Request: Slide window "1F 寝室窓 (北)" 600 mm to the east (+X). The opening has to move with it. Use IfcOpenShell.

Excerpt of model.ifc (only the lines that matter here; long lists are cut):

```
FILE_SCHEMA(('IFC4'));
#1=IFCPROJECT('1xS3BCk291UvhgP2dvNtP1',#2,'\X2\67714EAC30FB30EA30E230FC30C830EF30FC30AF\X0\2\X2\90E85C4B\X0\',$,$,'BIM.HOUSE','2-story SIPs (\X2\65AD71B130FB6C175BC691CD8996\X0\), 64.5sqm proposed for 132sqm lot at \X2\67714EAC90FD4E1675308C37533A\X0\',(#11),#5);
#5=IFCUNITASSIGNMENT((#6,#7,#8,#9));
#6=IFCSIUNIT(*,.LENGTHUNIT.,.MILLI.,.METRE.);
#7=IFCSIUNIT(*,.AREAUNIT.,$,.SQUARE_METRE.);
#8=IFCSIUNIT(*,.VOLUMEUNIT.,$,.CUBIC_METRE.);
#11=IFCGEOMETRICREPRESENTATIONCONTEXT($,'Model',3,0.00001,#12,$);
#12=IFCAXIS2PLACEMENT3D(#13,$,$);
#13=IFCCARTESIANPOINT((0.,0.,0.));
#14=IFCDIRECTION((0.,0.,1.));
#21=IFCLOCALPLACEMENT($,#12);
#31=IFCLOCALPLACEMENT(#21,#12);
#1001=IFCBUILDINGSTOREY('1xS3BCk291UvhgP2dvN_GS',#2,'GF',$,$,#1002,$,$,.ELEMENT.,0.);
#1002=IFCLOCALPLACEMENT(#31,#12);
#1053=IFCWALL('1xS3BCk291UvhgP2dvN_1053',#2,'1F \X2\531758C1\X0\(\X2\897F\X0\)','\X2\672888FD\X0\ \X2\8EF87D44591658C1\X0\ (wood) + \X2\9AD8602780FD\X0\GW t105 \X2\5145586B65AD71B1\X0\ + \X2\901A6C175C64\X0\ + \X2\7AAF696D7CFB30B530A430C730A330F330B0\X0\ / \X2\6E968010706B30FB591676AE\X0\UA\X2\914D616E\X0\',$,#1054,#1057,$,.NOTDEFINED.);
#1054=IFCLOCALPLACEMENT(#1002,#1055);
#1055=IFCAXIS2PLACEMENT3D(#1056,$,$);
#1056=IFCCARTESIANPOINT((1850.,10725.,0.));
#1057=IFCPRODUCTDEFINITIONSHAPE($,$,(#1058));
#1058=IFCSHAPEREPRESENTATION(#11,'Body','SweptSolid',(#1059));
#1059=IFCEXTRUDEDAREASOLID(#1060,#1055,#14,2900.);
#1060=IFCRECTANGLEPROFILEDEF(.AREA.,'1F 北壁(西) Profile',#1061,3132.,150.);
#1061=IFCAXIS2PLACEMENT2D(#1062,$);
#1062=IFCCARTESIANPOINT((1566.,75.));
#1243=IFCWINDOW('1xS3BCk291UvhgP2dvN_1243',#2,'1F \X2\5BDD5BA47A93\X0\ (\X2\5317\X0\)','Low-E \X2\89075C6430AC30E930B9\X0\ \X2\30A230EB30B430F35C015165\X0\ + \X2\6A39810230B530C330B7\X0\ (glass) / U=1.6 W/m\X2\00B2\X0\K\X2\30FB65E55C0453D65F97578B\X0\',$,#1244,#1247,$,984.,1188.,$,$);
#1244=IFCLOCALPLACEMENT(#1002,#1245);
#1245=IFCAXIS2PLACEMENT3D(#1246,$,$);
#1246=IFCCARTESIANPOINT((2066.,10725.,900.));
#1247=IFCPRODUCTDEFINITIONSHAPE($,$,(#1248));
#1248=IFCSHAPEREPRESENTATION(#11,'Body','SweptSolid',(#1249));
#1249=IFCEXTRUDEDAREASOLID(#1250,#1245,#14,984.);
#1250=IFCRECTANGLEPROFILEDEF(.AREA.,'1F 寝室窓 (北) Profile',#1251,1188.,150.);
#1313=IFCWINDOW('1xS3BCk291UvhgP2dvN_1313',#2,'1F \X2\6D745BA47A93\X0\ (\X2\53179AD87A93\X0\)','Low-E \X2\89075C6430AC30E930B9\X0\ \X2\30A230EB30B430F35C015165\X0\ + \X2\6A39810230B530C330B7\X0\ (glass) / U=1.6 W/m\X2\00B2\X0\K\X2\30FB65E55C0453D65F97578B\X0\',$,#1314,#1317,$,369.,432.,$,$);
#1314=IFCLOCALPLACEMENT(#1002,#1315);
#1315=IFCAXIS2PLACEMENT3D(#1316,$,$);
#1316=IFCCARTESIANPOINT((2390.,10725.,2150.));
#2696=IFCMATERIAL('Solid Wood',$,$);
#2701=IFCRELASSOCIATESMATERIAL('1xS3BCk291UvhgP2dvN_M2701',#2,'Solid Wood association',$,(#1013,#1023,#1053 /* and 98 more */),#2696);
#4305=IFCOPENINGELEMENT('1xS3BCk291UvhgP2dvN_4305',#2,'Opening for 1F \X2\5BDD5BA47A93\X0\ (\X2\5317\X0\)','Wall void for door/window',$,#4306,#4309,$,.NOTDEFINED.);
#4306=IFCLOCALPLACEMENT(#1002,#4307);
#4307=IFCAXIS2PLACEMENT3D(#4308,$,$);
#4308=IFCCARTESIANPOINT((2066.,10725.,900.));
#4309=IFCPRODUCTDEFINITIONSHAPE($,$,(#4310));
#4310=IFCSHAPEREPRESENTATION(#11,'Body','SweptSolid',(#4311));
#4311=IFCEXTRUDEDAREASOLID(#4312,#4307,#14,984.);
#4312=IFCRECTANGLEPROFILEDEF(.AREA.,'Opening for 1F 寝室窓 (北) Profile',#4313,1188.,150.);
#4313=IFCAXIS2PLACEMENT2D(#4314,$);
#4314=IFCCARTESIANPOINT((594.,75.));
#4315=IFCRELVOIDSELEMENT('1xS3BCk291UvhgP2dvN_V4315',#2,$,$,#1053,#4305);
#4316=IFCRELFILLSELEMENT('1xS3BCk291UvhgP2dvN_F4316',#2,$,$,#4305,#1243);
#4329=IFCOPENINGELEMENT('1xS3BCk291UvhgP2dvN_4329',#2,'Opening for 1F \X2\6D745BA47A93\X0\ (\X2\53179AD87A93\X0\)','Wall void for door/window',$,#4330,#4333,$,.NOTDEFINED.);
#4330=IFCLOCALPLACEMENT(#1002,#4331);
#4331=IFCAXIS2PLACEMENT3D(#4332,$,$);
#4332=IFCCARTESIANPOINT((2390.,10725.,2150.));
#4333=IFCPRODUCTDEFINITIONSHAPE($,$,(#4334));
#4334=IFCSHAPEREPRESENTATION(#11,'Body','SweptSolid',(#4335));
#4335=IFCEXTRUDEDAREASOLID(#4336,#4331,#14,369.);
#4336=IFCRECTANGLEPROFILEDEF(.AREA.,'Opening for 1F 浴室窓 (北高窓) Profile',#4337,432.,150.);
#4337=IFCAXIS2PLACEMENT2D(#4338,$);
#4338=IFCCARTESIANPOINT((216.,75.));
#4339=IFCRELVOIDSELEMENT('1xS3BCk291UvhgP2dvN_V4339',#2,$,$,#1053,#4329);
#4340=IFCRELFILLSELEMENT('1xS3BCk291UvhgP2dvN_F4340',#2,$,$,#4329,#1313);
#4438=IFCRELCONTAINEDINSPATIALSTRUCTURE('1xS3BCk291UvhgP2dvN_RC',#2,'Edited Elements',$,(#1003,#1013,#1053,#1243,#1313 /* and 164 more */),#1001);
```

```python
import ifcopenshell
import ifcopenshell.api.geometry
import ifcopenshell.util.placement

model = ifcopenshell.open("model.ifc")

window = model.by_guid("1xS3BCk291UvhgP2dvN_1243")
opening = window.FillsVoids[0].RelatingOpeningElement
wall = opening.VoidsElements[0].RelatingBuildingElement

wall_matrix = ifcopenshell.util.placement.get_local_placement(wall.ObjectPlacement)
shift = wall_matrix[:3, 0] * 600.0
before = ifcopenshell.util.placement.get_local_placement(window.ObjectPlacement)[:3, 3].copy()

# The window is not placed relative to its opening, so move both.
for product in (opening, window):
    matrix = ifcopenshell.util.placement.get_local_placement(product.ObjectPlacement)
    matrix[:3, 3] += shift
    ifcopenshell.api.geometry.edit_object_placement(model, product=product, matrix=matrix, is_si=False)

after = ifcopenshell.util.placement.get_local_placement(window.ObjectPlacement)[:3, 3]
print("window moved by", (after - before).round(3) + 0.0)

model.write("model-out.ifc")
```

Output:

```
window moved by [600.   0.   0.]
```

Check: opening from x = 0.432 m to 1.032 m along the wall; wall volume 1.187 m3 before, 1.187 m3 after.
